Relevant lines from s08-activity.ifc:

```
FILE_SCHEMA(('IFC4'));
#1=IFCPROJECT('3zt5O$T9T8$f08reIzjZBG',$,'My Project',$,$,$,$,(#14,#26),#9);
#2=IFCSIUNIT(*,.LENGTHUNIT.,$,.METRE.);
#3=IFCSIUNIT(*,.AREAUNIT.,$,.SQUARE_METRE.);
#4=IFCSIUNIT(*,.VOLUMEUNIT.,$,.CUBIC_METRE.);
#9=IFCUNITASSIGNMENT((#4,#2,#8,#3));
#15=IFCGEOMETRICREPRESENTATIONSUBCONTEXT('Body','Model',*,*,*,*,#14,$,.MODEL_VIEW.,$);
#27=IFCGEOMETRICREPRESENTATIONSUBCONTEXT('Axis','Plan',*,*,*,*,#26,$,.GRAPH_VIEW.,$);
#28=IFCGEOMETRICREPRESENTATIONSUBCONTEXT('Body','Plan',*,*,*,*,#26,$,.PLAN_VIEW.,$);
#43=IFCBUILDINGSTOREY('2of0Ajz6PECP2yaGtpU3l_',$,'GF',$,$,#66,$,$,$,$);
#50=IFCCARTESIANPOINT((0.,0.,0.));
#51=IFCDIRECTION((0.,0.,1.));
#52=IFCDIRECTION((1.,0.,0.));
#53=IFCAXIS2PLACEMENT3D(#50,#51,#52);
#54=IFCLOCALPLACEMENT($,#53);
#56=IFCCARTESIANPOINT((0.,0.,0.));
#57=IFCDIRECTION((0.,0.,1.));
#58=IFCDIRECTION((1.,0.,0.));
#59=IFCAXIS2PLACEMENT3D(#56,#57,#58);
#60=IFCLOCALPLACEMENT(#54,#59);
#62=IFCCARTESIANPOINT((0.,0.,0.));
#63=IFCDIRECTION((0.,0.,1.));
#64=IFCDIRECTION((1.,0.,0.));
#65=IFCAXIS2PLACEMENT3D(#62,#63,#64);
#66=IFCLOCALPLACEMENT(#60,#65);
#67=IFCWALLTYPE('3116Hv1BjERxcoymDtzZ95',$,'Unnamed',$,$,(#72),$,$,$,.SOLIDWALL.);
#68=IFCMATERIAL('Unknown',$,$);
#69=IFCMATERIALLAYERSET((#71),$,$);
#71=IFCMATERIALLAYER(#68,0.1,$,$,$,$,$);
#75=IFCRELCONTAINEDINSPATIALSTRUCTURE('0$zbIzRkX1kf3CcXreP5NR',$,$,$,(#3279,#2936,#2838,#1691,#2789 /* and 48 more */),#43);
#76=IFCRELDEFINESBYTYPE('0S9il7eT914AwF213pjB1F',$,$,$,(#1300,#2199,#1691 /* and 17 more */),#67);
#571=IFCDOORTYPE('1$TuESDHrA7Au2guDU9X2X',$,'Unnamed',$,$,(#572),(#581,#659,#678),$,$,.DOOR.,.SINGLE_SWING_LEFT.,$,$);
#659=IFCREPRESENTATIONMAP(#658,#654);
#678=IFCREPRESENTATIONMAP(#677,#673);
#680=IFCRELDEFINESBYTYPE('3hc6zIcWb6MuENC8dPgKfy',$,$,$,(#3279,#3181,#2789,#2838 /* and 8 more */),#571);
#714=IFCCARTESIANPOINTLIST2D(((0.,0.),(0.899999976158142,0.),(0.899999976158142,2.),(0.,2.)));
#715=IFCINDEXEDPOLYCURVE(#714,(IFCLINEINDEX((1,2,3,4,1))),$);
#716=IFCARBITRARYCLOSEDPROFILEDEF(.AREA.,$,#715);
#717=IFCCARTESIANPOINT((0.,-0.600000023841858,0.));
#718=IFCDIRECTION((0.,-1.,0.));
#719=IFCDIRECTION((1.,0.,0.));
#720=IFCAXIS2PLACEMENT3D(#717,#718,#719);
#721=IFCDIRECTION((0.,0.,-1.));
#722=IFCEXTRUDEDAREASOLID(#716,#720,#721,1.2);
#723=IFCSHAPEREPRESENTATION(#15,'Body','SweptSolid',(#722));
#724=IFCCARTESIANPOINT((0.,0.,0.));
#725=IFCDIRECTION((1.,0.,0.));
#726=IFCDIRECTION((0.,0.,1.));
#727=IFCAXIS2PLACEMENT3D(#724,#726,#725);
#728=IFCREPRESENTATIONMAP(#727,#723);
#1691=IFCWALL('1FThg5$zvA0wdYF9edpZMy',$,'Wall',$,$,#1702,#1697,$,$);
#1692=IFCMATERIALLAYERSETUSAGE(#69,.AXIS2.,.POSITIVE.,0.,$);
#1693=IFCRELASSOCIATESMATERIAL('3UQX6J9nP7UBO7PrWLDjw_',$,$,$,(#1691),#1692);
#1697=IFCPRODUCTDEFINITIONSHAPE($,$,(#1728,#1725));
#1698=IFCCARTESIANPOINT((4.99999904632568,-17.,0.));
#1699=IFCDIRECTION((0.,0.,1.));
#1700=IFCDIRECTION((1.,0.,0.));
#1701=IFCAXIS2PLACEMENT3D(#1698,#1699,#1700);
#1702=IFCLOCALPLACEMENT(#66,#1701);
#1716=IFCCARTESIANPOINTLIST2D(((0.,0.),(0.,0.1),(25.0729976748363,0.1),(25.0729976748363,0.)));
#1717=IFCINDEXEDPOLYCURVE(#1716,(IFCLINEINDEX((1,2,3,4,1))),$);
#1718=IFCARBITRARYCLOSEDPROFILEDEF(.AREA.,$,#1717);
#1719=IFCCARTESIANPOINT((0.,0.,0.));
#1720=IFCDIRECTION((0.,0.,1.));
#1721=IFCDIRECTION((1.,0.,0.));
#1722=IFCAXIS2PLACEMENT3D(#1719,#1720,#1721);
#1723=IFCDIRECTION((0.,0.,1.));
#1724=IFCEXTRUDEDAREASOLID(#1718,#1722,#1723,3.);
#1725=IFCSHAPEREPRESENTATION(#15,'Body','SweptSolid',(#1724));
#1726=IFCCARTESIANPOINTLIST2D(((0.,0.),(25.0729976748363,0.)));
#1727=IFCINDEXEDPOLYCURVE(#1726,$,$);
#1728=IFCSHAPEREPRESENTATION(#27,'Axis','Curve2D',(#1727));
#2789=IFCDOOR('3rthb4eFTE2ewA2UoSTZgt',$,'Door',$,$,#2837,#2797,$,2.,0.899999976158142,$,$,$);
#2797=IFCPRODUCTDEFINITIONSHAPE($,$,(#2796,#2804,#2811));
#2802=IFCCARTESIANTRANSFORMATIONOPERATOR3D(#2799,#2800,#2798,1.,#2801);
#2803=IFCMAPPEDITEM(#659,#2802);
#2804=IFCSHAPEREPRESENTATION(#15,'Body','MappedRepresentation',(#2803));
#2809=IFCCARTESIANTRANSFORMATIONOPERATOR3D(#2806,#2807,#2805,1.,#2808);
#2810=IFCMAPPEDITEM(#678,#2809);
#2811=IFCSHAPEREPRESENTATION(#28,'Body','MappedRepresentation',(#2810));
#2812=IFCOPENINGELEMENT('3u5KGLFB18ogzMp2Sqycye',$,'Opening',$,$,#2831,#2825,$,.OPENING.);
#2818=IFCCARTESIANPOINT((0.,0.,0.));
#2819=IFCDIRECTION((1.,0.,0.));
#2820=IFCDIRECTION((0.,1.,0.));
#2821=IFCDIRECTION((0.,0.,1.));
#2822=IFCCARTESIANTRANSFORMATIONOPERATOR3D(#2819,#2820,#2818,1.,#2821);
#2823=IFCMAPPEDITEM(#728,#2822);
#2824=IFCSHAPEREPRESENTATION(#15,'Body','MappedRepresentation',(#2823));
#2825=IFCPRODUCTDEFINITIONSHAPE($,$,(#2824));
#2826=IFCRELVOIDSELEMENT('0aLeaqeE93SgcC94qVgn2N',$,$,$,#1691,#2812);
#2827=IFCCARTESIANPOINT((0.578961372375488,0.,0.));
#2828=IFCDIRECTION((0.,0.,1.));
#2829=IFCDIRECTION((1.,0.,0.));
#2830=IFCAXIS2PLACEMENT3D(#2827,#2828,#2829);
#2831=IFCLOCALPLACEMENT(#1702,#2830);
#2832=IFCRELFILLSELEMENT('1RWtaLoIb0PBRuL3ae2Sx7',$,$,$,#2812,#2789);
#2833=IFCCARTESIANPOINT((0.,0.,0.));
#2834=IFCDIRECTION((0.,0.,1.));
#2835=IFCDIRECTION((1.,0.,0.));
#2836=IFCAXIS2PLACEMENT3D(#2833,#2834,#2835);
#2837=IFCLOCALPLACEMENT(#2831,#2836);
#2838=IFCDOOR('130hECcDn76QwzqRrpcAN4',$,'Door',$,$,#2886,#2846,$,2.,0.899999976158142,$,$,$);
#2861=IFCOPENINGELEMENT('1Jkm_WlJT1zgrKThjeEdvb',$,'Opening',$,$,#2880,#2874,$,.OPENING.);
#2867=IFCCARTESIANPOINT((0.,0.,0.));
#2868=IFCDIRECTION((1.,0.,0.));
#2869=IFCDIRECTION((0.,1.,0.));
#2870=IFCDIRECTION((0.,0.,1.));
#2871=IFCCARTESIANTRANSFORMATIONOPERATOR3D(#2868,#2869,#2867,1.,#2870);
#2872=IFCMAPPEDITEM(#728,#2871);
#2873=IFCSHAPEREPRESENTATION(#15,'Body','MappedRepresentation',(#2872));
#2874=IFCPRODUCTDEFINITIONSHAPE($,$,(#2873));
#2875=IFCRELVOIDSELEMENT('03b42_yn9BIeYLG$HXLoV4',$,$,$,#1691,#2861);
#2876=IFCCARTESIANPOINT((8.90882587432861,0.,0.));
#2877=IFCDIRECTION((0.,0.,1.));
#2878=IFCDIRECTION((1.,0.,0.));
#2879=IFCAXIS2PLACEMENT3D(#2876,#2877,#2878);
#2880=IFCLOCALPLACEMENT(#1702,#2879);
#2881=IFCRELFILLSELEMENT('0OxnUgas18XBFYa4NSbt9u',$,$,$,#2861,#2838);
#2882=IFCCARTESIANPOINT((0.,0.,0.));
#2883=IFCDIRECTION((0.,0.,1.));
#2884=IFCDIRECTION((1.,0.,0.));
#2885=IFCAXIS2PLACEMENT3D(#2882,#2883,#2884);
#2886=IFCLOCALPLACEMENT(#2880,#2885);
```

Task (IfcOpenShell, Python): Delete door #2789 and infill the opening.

```python
import ifcopenshell
import ifcopenshell.api.feature
import ifcopenshell.api.root
import ifcopenshell.geom
import ifcopenshell.util.shape

model = ifcopenshell.open("s08-activity.ifc")
settings = ifcopenshell.geom.settings()


def volume(element):
    """Net volume in cubic metres, openings subtracted."""
    shape = ifcopenshell.geom.create_shape(settings, element)
    return ifcopenshell.util.shape.get_volume(shape.geometry)


door = model.by_guid("3rthb4eFTE2ewA2UoSTZgt")
opening = door.FillsVoids[0].RelatingOpeningElement
wall = opening.VoidsElements[0].RelatingBuildingElement
before = volume(wall)

ifcopenshell.api.root.remove_product(model, product=door)
ifcopenshell.api.feature.remove_feature(model, feature=opening)

after = volume(wall)

print(f"wall volume {before:.3f} -> {after:.3f} m3")

model.write("s08-activity_v2.ifc")
```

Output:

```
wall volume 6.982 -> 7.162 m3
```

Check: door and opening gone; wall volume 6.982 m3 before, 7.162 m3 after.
